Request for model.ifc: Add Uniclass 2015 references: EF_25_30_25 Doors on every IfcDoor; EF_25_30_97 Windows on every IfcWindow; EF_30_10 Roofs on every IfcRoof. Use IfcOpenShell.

First a look at what the model holds.

```python
import ifcopenshell

model = ifcopenshell.open("model.ifc")
print(model.schema)
print("classifications:", [c.Name for c in model.by_type("IfcClassification")])
for ifc_class in ("IfcDoor", "IfcRoof", "IfcStair", "IfcWall", "IfcWindow"):
    print(ifc_class, len(model.by_type(ifc_class)))
```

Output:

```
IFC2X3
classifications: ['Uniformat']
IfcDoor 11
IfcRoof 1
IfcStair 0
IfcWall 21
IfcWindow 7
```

```python
import ifcopenshell
import ifcopenshell.api.classification

model = ifcopenshell.open("model.ifc")

# IFC2X3 requires Source and Edition and has no link from the project to the system.
system = model.create_entity("IfcClassification", Source="NBS", Edition="2015", Name="Uniclass 2015")

codes = {
    "IfcDoor": ("EF_25_30_25", "Doors"),
    "IfcWindow": ("EF_25_30_97", "Windows"),
    "IfcRoof": ("EF_30_10", "Roofs"),
}
for ifc_class, (code, name) in codes.items():
    products = model.by_type(ifc_class)
    ifcopenshell.api.classification.add_reference(
        model, products=products, classification=system, identification=code, name=name
    )
    print(code, len(products))

model.write("model_edited.ifc")
```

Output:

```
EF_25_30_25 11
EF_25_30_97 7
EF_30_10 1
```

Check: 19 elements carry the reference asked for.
